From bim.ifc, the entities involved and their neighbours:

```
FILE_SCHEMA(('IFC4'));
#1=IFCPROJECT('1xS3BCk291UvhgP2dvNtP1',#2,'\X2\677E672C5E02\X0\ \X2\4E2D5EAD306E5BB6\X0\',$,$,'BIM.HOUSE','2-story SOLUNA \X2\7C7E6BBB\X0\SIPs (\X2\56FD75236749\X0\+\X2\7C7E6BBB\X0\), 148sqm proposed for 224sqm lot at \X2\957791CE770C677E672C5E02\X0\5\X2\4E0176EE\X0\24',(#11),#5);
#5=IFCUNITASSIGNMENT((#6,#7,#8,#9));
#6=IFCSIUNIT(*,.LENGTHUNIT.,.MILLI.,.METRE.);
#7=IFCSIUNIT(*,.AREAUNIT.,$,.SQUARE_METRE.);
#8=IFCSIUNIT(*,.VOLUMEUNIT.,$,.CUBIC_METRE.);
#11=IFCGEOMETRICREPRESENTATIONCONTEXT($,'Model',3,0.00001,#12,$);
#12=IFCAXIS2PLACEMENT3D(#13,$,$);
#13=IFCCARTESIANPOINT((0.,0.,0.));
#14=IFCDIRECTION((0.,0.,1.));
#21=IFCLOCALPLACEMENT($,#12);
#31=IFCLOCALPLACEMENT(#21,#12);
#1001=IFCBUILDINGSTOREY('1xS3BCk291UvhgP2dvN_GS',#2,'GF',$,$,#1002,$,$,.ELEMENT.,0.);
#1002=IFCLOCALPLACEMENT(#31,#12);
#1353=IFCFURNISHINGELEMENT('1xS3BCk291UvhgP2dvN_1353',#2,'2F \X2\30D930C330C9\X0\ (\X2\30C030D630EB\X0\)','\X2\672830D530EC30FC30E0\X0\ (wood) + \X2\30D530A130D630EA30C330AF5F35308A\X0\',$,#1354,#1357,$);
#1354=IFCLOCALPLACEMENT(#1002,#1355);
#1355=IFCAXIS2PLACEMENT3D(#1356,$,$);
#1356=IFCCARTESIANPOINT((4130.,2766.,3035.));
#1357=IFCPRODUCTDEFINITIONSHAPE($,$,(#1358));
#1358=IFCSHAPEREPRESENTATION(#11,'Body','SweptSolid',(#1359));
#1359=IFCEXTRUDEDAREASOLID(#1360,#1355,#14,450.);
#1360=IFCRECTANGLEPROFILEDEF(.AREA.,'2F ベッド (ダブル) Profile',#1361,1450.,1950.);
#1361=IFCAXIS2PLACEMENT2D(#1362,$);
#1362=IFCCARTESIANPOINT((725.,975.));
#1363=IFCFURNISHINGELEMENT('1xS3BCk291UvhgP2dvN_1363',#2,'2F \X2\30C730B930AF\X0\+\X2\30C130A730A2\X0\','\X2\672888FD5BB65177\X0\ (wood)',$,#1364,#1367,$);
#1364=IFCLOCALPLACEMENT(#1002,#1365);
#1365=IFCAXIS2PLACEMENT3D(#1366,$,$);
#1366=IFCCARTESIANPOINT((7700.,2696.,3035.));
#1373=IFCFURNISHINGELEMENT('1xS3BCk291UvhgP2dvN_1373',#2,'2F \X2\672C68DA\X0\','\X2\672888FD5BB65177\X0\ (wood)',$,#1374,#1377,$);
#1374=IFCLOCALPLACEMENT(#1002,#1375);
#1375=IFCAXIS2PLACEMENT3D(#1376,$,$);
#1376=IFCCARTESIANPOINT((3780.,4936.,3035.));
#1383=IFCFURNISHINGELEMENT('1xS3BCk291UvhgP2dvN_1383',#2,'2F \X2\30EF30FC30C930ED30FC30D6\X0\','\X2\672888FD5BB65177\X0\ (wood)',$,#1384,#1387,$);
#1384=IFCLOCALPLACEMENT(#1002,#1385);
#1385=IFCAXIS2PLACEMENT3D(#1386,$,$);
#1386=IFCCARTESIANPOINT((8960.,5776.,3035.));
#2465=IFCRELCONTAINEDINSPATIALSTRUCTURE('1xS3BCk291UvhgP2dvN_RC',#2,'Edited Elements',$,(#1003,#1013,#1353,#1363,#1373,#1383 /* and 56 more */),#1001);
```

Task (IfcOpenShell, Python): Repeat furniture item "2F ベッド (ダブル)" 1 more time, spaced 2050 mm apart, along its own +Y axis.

```python
import ifcopenshell
import ifcopenshell.api.geometry
import ifcopenshell.api.root
import ifcopenshell.util.element
import ifcopenshell.util.placement

model = ifcopenshell.open("bim.ifc")


def reuse_history(source, copy):
    """copy_class also copies each property set's owner history, people and application; keep the originals."""
    for rel in copy.IsDefinedBy:
        if rel.is_a("IfcRelDefinesByProperties") and (history := rel.RelatingPropertyDefinition.OwnerHistory):
            rel.RelatingPropertyDefinition.OwnerHistory = source.OwnerHistory
            ifcopenshell.util.element.remove_deep2(model, history)


source = model.by_guid("1xS3BCk291UvhgP2dvN_1353")
base = ifcopenshell.util.placement.get_local_placement(source.ObjectPlacement)
step = base[:3, 1] * 2050.0

for i in range(1, 2):
    copy = ifcopenshell.api.root.copy_class(model, product=source)
    copy.Representation = ifcopenshell.util.element.copy_deep(
        model, source.Representation, exclude=["IfcGeometricRepresentationContext", "IfcRepresentationMap"]
    )
    reuse_history(source, copy)
    matrix = base.copy()
    matrix[:3, 3] += i * step
    print("added at", matrix[:3, 3].round(3) + 0.0)
    ifcopenshell.api.geometry.edit_object_placement(model, product=copy, matrix=matrix, is_si=False)

model.write("bim_updated.ifc")
```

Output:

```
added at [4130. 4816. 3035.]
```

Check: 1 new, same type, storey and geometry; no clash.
